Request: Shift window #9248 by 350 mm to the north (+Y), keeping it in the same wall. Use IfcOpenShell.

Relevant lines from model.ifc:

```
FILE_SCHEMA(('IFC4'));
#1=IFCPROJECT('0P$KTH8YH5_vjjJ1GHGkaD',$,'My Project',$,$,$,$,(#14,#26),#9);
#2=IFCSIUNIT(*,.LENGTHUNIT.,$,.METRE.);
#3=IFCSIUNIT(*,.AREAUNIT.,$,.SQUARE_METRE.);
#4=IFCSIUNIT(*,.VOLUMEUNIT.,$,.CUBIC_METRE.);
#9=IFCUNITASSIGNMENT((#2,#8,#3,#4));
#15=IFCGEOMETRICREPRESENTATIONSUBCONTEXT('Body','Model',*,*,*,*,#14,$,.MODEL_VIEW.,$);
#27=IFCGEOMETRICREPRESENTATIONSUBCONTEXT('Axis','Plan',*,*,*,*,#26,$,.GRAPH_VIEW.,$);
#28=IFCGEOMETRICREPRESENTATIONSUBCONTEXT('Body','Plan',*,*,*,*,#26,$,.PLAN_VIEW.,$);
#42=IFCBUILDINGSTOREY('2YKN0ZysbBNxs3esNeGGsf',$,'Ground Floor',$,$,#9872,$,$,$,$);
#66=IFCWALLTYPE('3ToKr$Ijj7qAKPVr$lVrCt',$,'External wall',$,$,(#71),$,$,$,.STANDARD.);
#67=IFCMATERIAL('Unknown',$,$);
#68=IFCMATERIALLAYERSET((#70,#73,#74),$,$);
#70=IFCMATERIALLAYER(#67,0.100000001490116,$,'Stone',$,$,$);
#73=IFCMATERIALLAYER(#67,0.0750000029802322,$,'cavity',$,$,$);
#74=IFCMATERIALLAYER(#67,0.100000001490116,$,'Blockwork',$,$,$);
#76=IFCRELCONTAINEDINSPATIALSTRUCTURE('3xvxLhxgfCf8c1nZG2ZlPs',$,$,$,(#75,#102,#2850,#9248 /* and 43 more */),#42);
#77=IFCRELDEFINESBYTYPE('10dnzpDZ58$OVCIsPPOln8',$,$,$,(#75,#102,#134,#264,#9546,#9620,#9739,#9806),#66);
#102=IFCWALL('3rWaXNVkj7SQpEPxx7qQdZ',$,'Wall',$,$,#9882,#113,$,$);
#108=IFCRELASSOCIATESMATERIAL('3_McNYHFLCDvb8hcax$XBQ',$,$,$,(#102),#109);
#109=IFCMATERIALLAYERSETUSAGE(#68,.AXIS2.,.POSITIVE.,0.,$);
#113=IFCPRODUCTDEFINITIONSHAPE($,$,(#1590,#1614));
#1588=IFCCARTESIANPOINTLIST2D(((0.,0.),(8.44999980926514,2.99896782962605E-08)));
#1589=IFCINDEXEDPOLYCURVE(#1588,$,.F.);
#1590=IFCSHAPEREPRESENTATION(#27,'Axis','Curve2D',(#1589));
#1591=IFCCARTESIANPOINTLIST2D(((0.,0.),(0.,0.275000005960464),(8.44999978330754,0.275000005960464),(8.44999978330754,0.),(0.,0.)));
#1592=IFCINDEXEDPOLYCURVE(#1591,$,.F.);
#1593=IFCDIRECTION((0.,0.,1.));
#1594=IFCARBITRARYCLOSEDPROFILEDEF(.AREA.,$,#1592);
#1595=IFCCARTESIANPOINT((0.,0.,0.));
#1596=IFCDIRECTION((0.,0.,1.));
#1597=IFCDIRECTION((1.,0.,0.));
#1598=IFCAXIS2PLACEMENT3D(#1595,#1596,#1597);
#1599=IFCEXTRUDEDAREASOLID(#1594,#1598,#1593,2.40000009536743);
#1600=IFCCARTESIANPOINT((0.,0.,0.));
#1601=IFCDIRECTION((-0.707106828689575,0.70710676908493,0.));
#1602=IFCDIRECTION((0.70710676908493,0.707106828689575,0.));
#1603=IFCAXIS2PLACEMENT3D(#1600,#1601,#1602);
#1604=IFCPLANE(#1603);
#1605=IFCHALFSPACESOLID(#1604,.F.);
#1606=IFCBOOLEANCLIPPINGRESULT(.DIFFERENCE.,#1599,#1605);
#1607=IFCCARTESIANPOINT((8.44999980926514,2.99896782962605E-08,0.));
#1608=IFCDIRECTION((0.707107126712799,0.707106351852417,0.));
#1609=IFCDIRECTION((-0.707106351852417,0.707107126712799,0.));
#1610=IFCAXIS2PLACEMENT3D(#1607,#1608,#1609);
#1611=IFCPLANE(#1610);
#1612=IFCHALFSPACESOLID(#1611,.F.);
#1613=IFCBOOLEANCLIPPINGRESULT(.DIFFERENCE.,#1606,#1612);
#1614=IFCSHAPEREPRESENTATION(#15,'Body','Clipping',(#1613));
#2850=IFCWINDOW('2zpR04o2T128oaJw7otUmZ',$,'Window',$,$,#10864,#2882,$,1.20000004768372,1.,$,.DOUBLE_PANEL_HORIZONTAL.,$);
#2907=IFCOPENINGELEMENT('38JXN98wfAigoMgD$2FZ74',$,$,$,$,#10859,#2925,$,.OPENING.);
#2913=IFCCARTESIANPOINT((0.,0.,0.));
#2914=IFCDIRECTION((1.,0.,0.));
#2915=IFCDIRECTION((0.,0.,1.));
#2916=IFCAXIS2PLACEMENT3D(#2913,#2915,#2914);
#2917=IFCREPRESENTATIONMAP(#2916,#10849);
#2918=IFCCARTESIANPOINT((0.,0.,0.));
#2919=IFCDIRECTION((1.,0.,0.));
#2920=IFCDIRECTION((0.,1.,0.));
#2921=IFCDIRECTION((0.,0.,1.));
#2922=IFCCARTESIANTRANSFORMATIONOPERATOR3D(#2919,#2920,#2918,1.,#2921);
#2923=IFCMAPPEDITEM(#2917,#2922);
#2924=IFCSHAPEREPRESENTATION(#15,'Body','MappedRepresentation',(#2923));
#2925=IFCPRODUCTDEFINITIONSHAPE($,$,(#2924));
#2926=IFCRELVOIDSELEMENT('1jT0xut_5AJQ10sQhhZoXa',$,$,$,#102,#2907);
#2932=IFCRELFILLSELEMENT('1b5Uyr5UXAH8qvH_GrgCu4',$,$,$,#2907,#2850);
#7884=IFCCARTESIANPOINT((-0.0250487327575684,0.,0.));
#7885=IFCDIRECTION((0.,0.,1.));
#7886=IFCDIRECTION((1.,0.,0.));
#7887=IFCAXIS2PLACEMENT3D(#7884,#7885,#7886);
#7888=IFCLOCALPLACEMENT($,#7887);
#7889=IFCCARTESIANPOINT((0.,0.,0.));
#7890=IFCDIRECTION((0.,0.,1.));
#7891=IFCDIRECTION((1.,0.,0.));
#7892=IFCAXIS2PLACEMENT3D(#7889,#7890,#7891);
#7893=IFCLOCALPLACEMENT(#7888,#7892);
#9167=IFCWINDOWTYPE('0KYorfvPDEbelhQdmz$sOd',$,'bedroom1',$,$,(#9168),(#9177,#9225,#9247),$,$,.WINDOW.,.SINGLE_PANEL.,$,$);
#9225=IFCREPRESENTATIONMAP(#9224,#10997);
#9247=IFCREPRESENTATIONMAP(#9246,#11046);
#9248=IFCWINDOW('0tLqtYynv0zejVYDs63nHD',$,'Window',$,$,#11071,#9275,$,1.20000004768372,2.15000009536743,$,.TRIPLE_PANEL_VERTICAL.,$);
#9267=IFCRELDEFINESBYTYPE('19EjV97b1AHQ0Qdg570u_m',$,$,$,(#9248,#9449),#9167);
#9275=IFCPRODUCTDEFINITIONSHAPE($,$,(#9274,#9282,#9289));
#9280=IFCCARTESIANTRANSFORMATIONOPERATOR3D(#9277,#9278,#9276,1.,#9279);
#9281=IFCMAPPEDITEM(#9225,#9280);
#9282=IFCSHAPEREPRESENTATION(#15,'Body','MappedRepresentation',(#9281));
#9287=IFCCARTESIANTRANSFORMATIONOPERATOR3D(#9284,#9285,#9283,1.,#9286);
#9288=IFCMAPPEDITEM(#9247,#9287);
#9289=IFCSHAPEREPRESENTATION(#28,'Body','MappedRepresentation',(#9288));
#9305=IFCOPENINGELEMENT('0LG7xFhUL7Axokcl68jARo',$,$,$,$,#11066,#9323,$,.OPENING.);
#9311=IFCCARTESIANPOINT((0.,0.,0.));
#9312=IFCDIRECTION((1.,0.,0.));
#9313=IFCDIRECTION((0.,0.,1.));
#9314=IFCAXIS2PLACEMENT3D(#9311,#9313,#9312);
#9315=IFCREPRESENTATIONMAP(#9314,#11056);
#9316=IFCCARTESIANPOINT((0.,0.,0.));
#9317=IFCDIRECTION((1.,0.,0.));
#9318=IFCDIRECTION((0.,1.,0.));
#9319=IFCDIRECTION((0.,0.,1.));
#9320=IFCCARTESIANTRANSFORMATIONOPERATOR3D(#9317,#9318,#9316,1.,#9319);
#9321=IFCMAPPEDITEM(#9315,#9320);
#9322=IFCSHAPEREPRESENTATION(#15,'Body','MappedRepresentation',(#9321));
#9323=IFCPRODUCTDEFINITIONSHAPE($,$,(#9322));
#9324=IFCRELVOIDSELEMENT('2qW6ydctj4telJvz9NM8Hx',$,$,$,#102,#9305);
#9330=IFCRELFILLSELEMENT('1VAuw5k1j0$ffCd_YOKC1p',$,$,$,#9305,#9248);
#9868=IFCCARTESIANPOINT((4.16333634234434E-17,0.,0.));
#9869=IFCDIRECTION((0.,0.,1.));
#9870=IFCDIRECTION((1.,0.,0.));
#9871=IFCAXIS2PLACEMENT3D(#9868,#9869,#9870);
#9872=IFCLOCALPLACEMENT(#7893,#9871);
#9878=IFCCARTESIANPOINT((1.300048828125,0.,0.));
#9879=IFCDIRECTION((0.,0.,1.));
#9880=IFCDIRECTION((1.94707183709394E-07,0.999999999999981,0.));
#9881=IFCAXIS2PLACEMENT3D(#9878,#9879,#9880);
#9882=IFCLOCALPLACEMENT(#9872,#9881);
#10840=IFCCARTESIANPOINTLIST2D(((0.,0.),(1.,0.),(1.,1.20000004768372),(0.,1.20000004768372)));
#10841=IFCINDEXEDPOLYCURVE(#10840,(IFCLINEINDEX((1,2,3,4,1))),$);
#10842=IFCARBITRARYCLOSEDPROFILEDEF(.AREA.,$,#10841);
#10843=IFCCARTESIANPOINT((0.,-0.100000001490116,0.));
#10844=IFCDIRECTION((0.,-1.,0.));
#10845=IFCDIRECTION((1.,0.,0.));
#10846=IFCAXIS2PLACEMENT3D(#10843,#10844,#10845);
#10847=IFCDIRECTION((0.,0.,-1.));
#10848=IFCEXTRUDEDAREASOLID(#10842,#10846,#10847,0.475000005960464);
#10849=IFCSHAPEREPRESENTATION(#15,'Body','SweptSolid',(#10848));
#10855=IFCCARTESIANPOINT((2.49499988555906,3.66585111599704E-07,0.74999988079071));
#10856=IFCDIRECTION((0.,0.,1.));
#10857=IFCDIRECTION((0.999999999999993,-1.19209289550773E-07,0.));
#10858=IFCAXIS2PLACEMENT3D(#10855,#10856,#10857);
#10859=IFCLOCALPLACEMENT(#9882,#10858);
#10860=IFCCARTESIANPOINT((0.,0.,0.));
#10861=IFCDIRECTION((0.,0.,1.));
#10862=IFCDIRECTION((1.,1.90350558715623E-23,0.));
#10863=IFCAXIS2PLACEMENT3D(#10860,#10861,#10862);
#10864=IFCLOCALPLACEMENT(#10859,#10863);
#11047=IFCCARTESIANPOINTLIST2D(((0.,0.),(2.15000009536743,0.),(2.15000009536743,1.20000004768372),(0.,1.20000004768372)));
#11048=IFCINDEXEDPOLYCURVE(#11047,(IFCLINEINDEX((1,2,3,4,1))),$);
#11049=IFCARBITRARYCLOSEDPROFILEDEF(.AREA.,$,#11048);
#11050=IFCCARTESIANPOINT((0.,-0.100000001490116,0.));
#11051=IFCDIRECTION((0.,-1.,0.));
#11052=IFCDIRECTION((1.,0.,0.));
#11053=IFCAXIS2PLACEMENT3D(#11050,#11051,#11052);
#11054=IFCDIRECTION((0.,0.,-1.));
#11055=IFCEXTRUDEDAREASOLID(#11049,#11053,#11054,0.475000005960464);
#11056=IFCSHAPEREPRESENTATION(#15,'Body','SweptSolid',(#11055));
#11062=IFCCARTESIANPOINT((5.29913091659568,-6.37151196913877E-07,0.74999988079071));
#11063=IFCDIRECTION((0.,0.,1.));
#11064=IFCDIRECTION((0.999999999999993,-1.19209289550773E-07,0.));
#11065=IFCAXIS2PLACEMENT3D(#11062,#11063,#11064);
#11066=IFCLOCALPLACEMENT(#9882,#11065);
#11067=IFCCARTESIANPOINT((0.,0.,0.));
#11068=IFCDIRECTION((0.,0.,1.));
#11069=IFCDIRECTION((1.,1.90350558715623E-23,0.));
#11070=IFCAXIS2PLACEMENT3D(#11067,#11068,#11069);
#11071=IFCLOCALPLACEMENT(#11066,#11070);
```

```python
import ifcopenshell
import ifcopenshell.api.geometry
import ifcopenshell.util.placement
import ifcopenshell.util.unit

model = ifcopenshell.open("model.ifc")
unit_scale = ifcopenshell.util.unit.calculate_unit_scale(model)

window = model.by_id(9248)
opening = window.FillsVoids[0].RelatingOpeningElement
wall = opening.VoidsElements[0].RelatingBuildingElement

wall_matrix = ifcopenshell.util.placement.get_local_placement(wall.ObjectPlacement)
shift = wall_matrix[:3, 0] * 0.35 / unit_scale
before = ifcopenshell.util.placement.get_local_placement(window.ObjectPlacement)[:3, 3].copy()

# The window is placed relative to its opening, so it follows when the opening moves.
matrix = ifcopenshell.util.placement.get_local_placement(opening.ObjectPlacement)
matrix[:3, 3] += shift
ifcopenshell.api.geometry.edit_object_placement(
    model, product=opening, matrix=matrix, is_si=False, should_transform_children=True
)

after = ifcopenshell.util.placement.get_local_placement(window.ObjectPlacement)[:3, 3]
print("window moved by", (after - before).round(3) + 0.0)

model.write("model_v2.ifc")
```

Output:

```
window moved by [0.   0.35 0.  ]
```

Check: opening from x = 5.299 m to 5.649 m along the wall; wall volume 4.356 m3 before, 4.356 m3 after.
